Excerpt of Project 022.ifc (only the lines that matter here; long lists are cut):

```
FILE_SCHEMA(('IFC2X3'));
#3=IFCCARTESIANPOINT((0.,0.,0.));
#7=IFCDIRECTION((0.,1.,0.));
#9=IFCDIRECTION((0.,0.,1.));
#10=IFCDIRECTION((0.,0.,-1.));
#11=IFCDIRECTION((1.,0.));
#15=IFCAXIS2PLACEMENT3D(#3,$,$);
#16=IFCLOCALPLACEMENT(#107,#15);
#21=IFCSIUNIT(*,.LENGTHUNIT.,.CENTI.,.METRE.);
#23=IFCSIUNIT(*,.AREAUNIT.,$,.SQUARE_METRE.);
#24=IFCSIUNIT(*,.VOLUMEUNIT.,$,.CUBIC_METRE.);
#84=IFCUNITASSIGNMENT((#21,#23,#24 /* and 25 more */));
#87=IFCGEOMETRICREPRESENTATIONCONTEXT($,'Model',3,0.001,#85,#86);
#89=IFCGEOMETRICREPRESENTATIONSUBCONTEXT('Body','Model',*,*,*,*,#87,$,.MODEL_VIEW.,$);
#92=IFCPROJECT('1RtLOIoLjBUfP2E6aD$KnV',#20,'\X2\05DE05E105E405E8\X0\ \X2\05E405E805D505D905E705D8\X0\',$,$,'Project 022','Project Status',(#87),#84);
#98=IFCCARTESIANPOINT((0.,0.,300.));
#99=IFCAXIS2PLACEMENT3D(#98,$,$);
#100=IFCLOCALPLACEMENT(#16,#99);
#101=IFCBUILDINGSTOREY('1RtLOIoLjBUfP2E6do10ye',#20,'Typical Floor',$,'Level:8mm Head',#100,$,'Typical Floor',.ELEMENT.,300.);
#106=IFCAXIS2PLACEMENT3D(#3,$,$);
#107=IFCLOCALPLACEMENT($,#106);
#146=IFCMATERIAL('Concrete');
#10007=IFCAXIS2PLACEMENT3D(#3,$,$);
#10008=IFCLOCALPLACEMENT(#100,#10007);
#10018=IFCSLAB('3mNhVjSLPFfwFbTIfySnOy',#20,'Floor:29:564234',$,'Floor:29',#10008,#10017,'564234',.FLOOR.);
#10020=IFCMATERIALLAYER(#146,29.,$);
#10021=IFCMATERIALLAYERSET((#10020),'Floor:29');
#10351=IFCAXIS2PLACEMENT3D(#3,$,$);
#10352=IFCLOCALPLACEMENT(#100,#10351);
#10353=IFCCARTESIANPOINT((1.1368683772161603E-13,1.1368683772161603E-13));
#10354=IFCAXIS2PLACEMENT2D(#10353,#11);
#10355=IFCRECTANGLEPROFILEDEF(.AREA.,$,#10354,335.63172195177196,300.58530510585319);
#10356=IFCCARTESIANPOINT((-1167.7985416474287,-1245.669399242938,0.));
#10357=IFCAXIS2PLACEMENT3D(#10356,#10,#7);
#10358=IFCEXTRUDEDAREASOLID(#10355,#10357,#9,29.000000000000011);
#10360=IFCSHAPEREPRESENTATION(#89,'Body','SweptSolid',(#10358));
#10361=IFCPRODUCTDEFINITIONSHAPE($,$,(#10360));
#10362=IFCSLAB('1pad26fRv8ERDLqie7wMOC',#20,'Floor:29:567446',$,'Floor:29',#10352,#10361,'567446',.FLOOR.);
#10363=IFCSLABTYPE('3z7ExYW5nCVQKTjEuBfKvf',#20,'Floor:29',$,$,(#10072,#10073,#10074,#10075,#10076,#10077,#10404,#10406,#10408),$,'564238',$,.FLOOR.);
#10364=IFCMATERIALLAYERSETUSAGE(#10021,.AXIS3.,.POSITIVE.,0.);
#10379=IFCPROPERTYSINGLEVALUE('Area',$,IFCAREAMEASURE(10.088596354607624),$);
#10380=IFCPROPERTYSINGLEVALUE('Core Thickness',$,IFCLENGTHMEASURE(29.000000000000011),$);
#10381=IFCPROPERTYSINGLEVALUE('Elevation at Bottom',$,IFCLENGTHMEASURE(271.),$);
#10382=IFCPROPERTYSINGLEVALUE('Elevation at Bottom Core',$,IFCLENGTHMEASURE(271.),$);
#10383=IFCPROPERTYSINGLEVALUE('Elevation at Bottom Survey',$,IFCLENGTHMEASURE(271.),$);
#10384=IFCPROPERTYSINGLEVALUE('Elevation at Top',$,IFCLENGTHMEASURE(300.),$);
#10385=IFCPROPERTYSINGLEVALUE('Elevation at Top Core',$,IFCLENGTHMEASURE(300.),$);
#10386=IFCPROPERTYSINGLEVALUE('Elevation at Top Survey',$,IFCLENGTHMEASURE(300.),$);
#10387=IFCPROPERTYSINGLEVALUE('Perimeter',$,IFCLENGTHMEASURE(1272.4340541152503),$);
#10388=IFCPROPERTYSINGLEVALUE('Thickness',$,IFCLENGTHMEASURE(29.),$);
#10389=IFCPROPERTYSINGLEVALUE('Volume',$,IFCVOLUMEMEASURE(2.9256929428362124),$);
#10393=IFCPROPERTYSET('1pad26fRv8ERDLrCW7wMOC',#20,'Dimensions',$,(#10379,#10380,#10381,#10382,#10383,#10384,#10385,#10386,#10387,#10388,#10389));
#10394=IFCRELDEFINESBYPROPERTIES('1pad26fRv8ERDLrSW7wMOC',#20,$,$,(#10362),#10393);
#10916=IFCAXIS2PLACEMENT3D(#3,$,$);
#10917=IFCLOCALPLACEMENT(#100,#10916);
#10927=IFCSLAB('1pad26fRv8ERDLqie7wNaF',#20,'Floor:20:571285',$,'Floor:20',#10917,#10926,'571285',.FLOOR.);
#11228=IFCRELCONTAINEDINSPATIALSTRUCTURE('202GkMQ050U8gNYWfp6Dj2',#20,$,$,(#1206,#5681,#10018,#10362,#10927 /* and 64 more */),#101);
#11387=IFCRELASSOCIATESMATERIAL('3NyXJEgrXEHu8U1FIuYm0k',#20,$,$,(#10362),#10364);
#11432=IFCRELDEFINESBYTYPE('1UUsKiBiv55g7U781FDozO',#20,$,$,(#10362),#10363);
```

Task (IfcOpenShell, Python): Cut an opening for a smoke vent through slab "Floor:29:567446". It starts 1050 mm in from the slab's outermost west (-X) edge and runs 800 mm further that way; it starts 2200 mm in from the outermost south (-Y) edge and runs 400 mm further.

```python
import numpy as np
import ifcopenshell
import ifcopenshell.api.feature
import ifcopenshell.api.geometry
import ifcopenshell.api.pset
import ifcopenshell.api.root
import ifcopenshell.geom
import ifcopenshell.util.element
import ifcopenshell.util.placement
import ifcopenshell.util.representation
import ifcopenshell.util.shape
import ifcopenshell.util.unit

model = ifcopenshell.open("Project 022.ifc")
unit_scale = ifcopenshell.util.unit.calculate_unit_scale(model)
area_scale = ifcopenshell.util.unit.calculate_unit_scale(model, "AREAUNIT")
volume_scale = ifcopenshell.util.unit.calculate_unit_scale(model, "VOLUMEUNIT")
settings = ifcopenshell.geom.settings()


def volume(element):
    """Net volume in cubic metres, openings subtracted."""
    shape = ifcopenshell.geom.create_shape(settings, element)
    return ifcopenshell.util.shape.get_volume(shape.geometry)


slab = model.by_id(10362)
before = volume(slab)

# Extent in the slab's own axes, in metres. The edges named are its -X and -Y sides.
slab_shape = ifcopenshell.geom.create_shape(settings, slab)
vertices = ifcopenshell.util.shape.get_vertices(slab_shape.geometry)
x_min, y_min, bottom = vertices.min(axis=0)
top = vertices[:, 2].max()

opening = ifcopenshell.api.root.create_entity(model, ifc_class="IfcOpeningElement", name="Smoke vent opening")
context = ifcopenshell.util.representation.get_context(model, "Model", "Body", "MODEL_VIEW")
width, depth = 0.8, 0.4
outline = [(0.0, 0.0), (width, 0.0), (width, depth), (0.0, depth), (0.0, 0.0)]
# Overshoot both faces by 50 mm so the cut is clean.
shape = ifcopenshell.api.geometry.add_slab_representation(
    model, context=context, depth=top - bottom + 0.1, polyline=outline
)
ifcopenshell.api.geometry.assign_representation(model, product=opening, representation=shape)

matrix = ifcopenshell.util.placement.get_local_placement(slab.ObjectPlacement)
matrix[:, 3] = matrix @ np.append(np.array([x_min + 1.05, y_min + 2.2, bottom - 0.05]) / unit_scale, 1.0)
ifcopenshell.api.geometry.edit_object_placement(model, product=opening, matrix=matrix, is_si=False)
ifcopenshell.api.feature.add_feature(model, feature=opening, element=slab)

after = volume(slab)

# Update the slab's stored quantities.
pset = model.by_id(ifcopenshell.util.element.get_pset(slab, "Dimensions", should_inherit=False)["id"])
ifcopenshell.api.pset.edit_pset(model, pset=pset, properties={
    "Area": model.create_entity("IfcAreaMeasure", after / (top - bottom) / area_scale),
    "Volume": model.create_entity("IfcVolumeMeasure", after / volume_scale),
})

print(f"slab volume {before:.3f} -> {after:.3f} m3")

model.write("Project 022_updated.ifc")
```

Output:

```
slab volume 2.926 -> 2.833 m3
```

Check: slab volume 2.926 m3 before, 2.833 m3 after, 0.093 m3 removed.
